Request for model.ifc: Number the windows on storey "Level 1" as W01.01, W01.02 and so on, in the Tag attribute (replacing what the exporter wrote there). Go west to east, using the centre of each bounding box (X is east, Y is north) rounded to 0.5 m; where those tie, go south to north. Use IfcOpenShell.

First a look at what the model holds.

```python
import ifcopenshell
import ifcopenshell.util.element
import ifcopenshell.util.placement

model = ifcopenshell.open("model.ifc")
print(model.schema)
storey = next(s for s in model.by_type("IfcBuildingStorey") if s.Name == "Level 1")
windows = [e for e in ifcopenshell.util.element.get_decomposition(storey) if e.is_a("IfcWindow")]
for e in sorted(windows, key=lambda e: e.id()):
    origin = ifcopenshell.util.placement.get_local_placement(e.ObjectPlacement)[:3, 3]
    print(e.id(), e.Tag, e.Name, origin.round(2) + 0.0, sep=" | ")
```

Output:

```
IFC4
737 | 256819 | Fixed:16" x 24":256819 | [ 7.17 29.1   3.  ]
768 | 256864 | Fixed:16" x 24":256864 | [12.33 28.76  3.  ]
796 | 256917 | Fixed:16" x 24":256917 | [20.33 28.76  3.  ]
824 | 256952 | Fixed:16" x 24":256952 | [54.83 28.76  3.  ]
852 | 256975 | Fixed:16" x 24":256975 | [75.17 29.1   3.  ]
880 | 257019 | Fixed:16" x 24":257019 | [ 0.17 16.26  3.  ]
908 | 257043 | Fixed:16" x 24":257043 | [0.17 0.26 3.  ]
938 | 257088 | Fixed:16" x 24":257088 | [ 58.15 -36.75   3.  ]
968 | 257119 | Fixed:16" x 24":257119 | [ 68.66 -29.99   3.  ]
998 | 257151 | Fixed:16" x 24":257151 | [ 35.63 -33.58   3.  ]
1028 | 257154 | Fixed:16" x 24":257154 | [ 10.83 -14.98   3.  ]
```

```python
import ifcopenshell
import ifcopenshell.geom
import ifcopenshell.util.element
import ifcopenshell.util.shape

model = ifcopenshell.open("model.ifc")
settings = ifcopenshell.geom.settings()
settings.set("use-world-coords", True)


def centre(element):
    shape = ifcopenshell.geom.create_shape(settings, element)
    return ifcopenshell.util.shape.get_bbox_centroid(shape.geometry)


storey = next(s for s in model.by_type("IfcBuildingStorey") if s.Name == "Level 1")
windows = [e for e in ifcopenshell.util.element.get_decomposition(storey) if e.is_a("IfcWindow")]

# Insertion points can sit at a corner or the storey origin, so sort by the geometry (in metres).
centres = {e: centre(e) for e in windows}
windows.sort(key=lambda e: (round(centres[e][0] / 0.5), centres[e][1]))

for i, e in enumerate(windows, start=1):
    number = f"W01.{i:02d}"
    e.Tag = number
    print(e.id(), number)

model.write("model_edited.ifc")
```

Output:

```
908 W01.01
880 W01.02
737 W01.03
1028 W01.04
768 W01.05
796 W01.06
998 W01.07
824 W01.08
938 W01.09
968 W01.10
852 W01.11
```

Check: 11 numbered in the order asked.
